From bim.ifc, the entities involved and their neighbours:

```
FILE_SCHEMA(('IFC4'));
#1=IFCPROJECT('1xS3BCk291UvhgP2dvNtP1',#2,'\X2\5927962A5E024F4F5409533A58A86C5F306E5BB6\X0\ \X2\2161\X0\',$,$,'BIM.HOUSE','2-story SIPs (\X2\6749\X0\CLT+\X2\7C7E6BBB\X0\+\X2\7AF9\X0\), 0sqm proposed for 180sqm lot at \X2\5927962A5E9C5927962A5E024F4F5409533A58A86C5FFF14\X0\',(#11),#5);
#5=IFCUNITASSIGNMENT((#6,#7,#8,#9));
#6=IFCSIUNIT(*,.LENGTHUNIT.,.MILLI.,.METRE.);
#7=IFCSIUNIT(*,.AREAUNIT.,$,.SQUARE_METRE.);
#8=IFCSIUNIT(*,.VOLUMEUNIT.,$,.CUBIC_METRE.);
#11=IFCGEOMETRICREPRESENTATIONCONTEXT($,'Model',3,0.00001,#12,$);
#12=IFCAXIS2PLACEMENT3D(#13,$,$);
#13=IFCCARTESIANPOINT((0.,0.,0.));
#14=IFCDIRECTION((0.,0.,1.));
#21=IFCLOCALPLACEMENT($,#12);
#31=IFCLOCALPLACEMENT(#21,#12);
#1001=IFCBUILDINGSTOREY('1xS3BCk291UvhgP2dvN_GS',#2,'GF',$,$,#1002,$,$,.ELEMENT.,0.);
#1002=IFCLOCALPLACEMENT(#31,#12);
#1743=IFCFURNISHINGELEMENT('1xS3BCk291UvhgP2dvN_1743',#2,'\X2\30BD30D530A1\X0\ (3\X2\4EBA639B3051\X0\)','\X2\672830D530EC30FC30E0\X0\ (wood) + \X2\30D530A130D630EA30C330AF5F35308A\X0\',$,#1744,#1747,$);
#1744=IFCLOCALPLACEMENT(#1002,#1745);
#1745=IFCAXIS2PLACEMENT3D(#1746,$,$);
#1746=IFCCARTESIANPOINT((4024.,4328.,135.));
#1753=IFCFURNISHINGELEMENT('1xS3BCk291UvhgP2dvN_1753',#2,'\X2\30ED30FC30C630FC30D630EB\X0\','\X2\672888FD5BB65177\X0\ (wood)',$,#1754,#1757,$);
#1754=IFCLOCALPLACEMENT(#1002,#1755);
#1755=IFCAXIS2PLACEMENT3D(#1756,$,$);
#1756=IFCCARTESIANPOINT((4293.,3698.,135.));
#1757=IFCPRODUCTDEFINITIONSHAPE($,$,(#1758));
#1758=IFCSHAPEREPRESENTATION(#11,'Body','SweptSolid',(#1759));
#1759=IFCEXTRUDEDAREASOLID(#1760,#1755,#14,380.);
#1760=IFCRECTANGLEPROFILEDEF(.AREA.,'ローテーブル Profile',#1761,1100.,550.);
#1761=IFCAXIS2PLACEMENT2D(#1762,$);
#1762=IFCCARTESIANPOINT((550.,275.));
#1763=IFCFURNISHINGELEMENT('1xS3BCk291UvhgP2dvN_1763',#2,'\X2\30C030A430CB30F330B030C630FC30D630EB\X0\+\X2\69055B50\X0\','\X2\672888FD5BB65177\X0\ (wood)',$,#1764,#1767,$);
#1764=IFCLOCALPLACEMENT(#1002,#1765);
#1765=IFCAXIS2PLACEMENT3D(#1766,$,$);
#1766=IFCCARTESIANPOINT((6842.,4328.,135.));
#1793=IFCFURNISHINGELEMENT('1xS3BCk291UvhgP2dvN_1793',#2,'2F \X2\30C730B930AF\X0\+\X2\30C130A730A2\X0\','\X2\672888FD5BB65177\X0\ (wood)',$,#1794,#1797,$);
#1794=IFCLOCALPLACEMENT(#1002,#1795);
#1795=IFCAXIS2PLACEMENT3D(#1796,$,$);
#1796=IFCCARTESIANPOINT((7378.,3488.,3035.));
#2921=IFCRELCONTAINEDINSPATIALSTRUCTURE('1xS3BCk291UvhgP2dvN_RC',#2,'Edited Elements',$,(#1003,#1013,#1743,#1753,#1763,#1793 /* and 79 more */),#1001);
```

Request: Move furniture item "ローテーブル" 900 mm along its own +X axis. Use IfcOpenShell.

```python
import ifcopenshell
import ifcopenshell.api.geometry
import ifcopenshell.util.placement
import ifcopenshell.util.unit

model = ifcopenshell.open("bim.ifc")
unit_scale = ifcopenshell.util.unit.calculate_unit_scale(model)

item = model.by_id(1753)
matrix = ifcopenshell.util.placement.get_local_placement(item.ObjectPlacement)
matrix[:3, 3] += matrix[:3, 0] * 0.9 / unit_scale
ifcopenshell.api.geometry.edit_object_placement(model, product=item, matrix=matrix, is_si=False)

print(ifcopenshell.util.placement.get_local_placement(item.ObjectPlacement).round(3) + 0.0)

model.write("bim-out.ifc")
```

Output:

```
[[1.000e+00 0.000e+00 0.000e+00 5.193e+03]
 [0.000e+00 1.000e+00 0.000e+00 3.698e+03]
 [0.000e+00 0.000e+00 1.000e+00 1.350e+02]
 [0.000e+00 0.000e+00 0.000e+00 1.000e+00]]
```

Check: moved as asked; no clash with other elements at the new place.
